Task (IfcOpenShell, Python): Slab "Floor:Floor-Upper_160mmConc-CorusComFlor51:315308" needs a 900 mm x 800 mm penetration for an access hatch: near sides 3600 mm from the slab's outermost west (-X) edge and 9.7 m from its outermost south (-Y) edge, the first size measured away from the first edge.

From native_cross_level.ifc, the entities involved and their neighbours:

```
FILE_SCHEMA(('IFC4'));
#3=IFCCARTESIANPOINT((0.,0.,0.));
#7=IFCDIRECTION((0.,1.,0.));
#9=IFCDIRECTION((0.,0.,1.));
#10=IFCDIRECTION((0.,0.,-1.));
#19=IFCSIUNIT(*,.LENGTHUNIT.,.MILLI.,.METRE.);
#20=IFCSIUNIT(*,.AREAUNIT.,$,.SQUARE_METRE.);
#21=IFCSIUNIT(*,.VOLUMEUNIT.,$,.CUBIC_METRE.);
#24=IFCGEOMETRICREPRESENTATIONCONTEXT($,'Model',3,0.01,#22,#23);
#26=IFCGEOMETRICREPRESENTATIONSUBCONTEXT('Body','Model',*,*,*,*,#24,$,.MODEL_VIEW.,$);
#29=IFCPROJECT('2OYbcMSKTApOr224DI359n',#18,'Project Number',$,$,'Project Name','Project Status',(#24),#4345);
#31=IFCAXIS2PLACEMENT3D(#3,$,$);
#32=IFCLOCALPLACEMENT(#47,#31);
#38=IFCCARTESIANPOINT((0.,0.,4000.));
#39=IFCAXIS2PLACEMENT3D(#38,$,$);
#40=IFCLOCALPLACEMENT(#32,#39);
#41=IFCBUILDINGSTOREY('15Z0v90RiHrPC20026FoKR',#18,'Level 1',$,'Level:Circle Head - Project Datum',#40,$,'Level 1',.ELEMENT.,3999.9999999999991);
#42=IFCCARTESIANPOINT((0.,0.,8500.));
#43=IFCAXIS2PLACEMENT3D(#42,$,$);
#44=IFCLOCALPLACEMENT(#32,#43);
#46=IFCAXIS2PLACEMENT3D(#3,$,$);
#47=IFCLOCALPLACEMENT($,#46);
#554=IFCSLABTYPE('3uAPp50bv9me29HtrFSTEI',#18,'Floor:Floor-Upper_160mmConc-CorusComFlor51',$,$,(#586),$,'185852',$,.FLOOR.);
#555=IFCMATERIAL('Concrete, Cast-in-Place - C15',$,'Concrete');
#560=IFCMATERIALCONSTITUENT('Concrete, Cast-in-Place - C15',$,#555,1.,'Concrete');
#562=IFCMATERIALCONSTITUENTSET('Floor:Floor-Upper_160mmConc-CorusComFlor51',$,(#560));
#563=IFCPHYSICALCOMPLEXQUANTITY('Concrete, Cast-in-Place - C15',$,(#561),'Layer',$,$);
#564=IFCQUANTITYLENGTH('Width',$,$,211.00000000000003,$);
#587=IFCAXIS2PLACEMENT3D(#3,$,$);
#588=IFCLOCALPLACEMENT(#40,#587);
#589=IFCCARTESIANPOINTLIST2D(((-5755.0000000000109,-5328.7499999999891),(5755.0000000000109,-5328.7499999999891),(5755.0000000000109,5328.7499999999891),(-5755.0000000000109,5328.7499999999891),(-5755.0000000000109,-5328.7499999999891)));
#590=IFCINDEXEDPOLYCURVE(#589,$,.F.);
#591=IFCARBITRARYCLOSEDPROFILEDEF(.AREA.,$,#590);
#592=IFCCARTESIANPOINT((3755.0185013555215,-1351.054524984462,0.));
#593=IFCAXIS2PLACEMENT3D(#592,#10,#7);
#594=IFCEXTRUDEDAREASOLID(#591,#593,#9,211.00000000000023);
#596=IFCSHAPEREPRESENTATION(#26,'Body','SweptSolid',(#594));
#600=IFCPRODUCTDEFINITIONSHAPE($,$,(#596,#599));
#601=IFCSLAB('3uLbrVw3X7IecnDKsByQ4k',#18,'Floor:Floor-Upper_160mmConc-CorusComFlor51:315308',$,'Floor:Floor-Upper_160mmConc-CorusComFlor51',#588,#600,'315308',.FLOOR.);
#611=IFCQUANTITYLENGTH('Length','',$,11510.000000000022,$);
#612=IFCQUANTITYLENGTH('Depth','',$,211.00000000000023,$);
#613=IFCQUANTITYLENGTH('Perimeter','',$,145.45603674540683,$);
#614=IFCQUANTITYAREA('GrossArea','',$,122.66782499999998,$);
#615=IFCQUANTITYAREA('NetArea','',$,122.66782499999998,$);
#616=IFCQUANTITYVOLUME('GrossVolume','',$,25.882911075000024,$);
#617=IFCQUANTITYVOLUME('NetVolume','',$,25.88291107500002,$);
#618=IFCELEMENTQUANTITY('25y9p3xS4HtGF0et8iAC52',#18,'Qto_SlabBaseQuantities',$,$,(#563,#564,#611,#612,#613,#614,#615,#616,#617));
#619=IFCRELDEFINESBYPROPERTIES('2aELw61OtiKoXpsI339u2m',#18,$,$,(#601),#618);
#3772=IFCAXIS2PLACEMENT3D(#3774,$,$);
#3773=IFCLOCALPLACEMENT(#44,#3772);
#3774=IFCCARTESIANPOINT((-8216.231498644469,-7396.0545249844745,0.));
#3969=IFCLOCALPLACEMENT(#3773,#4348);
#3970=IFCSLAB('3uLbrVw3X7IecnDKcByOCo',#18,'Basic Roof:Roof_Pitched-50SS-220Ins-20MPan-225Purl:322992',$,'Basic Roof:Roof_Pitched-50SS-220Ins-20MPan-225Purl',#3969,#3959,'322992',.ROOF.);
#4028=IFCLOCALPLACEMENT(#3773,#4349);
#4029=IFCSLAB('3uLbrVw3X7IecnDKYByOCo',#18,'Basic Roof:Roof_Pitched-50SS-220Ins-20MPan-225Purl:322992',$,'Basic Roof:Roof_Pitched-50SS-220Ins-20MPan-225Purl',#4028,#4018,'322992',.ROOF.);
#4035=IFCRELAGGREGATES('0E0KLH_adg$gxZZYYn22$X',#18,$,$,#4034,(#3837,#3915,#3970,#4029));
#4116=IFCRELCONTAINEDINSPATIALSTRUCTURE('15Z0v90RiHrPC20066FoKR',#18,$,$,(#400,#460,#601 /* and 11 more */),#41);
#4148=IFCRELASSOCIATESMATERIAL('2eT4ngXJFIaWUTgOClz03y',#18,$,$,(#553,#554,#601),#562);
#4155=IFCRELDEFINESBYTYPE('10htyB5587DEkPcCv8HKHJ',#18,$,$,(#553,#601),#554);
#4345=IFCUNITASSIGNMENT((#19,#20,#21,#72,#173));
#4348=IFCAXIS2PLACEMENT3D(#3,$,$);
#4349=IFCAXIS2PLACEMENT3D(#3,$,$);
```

```python
import numpy as np
import ifcopenshell
import ifcopenshell.api.feature
import ifcopenshell.api.geometry
import ifcopenshell.api.pset
import ifcopenshell.api.root
import ifcopenshell.geom
import ifcopenshell.util.element
import ifcopenshell.util.placement
import ifcopenshell.util.representation
import ifcopenshell.util.shape
import ifcopenshell.util.unit

model = ifcopenshell.open("native_cross_level.ifc")
unit_scale = ifcopenshell.util.unit.calculate_unit_scale(model)
area_scale = ifcopenshell.util.unit.calculate_unit_scale(model, "AREAUNIT")
volume_scale = ifcopenshell.util.unit.calculate_unit_scale(model, "VOLUMEUNIT")
settings = ifcopenshell.geom.settings()


def volume(element):
    """Net volume in cubic metres, openings subtracted."""
    shape = ifcopenshell.geom.create_shape(settings, element)
    return ifcopenshell.util.shape.get_volume(shape.geometry)


slab = model.by_id(601)
before = volume(slab)

# Extent in the slab's own axes, in metres. The edges named are its -X and -Y sides.
slab_shape = ifcopenshell.geom.create_shape(settings, slab)
vertices = ifcopenshell.util.shape.get_vertices(slab_shape.geometry)
x_min, y_min, bottom = vertices.min(axis=0)
top = vertices[:, 2].max()

opening = ifcopenshell.api.root.create_entity(model, ifc_class="IfcOpeningElement", name="Access hatch opening", predefined_type="OPENING")
context = ifcopenshell.util.representation.get_context(model, "Model", "Body", "MODEL_VIEW")
width, depth = 0.9, 0.8
outline = [(0.0, 0.0), (width, 0.0), (width, depth), (0.0, depth), (0.0, 0.0)]
# Overshoot both faces by 50 mm so the cut is clean.
shape = ifcopenshell.api.geometry.add_slab_representation(
    model, context=context, depth=top - bottom + 0.1, polyline=outline
)
ifcopenshell.api.geometry.assign_representation(model, product=opening, representation=shape)

matrix = ifcopenshell.util.placement.get_local_placement(slab.ObjectPlacement)
matrix[:, 3] = matrix @ np.append(np.array([x_min + 3.6, y_min + 9.7, bottom - 0.05]) / unit_scale, 1.0)
ifcopenshell.api.geometry.edit_object_placement(model, product=opening, matrix=matrix, is_si=False)
ifcopenshell.api.feature.add_feature(model, feature=opening, element=slab)

after = volume(slab)

# Update the slab's stored quantities.
qto = model.by_id(ifcopenshell.util.element.get_pset(slab, "Qto_SlabBaseQuantities", should_inherit=False)["id"])
ifcopenshell.api.pset.edit_qto(model, qto=qto, properties={
    "NetArea": after / (top - bottom) / area_scale,
    "NetVolume": after / volume_scale,
})

print(f"slab volume {before:.3f} -> {after:.3f} m3")

model.write("native_cross_level_edited.ifc")
```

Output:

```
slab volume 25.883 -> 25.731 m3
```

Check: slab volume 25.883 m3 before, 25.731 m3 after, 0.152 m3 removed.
